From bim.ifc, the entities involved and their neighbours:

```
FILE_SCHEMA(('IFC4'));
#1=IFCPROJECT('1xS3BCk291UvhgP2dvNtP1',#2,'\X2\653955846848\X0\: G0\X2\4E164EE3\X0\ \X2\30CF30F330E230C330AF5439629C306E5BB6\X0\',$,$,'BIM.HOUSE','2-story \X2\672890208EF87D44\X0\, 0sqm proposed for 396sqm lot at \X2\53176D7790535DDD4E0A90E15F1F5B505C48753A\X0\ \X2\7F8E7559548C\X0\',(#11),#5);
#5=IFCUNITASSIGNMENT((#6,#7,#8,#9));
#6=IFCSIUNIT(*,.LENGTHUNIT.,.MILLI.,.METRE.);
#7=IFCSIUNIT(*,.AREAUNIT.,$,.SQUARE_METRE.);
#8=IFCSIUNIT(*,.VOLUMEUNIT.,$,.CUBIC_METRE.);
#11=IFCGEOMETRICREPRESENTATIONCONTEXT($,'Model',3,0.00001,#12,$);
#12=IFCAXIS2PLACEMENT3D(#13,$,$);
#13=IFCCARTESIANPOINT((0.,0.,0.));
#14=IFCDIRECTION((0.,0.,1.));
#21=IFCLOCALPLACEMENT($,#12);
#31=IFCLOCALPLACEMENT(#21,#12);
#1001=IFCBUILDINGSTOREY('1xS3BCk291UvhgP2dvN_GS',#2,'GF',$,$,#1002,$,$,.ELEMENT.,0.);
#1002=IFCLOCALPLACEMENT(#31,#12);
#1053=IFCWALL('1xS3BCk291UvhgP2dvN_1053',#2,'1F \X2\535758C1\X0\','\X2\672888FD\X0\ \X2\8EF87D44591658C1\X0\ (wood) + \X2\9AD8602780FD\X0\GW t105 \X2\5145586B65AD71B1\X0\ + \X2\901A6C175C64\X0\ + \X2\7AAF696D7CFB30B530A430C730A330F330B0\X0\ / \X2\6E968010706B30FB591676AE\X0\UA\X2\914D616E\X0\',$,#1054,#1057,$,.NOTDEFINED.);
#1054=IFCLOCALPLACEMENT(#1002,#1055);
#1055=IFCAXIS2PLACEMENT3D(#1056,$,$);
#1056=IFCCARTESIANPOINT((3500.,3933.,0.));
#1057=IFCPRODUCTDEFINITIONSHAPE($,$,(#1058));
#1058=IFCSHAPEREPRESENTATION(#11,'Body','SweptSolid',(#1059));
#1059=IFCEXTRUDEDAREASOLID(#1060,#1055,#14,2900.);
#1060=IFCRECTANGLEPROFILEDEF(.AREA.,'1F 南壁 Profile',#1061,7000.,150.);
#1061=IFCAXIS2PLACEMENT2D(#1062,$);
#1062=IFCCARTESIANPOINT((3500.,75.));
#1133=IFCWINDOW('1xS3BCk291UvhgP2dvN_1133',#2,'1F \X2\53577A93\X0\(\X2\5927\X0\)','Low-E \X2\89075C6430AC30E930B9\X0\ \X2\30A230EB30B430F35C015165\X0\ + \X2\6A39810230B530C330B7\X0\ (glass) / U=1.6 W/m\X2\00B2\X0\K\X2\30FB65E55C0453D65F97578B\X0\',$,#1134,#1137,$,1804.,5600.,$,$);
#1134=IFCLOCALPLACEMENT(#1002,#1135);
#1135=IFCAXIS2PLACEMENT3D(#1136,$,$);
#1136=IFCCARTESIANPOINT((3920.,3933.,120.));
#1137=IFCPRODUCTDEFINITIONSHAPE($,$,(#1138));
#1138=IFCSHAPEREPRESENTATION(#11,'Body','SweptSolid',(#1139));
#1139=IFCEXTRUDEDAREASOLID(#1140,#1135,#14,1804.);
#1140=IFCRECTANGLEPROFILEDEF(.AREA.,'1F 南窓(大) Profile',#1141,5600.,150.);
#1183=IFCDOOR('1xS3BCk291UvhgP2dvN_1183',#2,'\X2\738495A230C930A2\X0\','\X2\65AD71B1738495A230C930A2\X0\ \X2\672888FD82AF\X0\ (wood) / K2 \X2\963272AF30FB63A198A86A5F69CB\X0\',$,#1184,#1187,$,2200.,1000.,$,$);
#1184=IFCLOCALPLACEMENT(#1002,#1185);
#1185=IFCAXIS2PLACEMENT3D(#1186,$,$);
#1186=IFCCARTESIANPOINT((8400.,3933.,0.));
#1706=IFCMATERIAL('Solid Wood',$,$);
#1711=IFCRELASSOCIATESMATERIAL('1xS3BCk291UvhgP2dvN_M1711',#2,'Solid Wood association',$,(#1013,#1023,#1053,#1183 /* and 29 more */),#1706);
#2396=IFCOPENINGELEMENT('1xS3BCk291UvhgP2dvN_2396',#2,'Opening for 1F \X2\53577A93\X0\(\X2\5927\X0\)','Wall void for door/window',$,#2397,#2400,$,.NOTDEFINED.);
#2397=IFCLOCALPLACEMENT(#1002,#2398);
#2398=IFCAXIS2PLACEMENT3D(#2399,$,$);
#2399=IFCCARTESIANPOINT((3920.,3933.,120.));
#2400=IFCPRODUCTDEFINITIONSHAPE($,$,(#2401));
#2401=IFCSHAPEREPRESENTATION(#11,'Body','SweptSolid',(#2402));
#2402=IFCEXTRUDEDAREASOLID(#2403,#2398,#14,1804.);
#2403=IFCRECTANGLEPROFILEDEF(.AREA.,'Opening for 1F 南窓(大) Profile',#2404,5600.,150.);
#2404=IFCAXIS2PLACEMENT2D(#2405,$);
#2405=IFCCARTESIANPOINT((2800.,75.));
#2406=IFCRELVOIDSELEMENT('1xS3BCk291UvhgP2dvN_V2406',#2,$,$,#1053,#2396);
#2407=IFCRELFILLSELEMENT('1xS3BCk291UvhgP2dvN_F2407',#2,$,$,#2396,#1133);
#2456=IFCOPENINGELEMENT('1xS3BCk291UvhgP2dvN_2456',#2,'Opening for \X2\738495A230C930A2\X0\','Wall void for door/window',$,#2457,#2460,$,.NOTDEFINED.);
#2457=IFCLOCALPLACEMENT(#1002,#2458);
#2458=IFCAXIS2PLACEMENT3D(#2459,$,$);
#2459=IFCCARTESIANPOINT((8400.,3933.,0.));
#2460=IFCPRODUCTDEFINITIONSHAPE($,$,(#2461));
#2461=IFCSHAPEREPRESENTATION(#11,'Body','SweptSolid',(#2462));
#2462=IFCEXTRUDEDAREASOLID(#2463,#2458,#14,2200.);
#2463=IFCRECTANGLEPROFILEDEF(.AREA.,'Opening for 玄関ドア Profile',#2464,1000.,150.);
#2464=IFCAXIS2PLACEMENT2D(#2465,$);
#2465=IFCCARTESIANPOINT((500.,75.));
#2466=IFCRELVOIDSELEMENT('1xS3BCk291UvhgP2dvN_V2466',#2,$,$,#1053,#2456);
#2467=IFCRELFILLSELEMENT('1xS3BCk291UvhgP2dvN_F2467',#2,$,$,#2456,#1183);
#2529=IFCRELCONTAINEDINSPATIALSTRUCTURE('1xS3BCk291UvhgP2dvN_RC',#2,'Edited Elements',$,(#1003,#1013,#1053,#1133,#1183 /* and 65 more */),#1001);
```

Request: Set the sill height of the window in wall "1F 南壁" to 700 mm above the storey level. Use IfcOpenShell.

```python
import numpy as np
import ifcopenshell
import ifcopenshell.api.geometry
import ifcopenshell.geom
import ifcopenshell.util.element
import ifcopenshell.util.placement
import ifcopenshell.util.shape
import ifcopenshell.util.unit

model = ifcopenshell.open("bim.ifc")
unit_scale = ifcopenshell.util.unit.calculate_unit_scale(model)

window = model.by_id(1133)
opening = window.FillsVoids[0].RelatingOpeningElement
storey = ifcopenshell.util.element.get_container(window, ifc_class="IfcBuildingStorey")
level = ifcopenshell.util.placement.get_local_placement(storey.ObjectPlacement)[2, 3]

# The opening's origin need not be at the sill, so measure its lowest point.
shape = ifcopenshell.geom.create_shape(ifcopenshell.geom.settings(), opening)
bottom = ifcopenshell.util.shape.get_shape_bottom_elevation(shape, shape.geometry) / unit_scale
dz = level + 0.7 / unit_scale - bottom

shift = np.array([0.0, 0.0, dz])
# The window is not placed relative to its opening, so move both.
for product in (opening, window):
    matrix = ifcopenshell.util.placement.get_local_placement(product.ObjectPlacement)
    matrix[:3, 3] += shift
    ifcopenshell.api.geometry.edit_object_placement(model, product=product, matrix=matrix, is_si=False)

print(f"moved by {dz * unit_scale:+.3f} m")

model.write("bim_updated.ifc")
```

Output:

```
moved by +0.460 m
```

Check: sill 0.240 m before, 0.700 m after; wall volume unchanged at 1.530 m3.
